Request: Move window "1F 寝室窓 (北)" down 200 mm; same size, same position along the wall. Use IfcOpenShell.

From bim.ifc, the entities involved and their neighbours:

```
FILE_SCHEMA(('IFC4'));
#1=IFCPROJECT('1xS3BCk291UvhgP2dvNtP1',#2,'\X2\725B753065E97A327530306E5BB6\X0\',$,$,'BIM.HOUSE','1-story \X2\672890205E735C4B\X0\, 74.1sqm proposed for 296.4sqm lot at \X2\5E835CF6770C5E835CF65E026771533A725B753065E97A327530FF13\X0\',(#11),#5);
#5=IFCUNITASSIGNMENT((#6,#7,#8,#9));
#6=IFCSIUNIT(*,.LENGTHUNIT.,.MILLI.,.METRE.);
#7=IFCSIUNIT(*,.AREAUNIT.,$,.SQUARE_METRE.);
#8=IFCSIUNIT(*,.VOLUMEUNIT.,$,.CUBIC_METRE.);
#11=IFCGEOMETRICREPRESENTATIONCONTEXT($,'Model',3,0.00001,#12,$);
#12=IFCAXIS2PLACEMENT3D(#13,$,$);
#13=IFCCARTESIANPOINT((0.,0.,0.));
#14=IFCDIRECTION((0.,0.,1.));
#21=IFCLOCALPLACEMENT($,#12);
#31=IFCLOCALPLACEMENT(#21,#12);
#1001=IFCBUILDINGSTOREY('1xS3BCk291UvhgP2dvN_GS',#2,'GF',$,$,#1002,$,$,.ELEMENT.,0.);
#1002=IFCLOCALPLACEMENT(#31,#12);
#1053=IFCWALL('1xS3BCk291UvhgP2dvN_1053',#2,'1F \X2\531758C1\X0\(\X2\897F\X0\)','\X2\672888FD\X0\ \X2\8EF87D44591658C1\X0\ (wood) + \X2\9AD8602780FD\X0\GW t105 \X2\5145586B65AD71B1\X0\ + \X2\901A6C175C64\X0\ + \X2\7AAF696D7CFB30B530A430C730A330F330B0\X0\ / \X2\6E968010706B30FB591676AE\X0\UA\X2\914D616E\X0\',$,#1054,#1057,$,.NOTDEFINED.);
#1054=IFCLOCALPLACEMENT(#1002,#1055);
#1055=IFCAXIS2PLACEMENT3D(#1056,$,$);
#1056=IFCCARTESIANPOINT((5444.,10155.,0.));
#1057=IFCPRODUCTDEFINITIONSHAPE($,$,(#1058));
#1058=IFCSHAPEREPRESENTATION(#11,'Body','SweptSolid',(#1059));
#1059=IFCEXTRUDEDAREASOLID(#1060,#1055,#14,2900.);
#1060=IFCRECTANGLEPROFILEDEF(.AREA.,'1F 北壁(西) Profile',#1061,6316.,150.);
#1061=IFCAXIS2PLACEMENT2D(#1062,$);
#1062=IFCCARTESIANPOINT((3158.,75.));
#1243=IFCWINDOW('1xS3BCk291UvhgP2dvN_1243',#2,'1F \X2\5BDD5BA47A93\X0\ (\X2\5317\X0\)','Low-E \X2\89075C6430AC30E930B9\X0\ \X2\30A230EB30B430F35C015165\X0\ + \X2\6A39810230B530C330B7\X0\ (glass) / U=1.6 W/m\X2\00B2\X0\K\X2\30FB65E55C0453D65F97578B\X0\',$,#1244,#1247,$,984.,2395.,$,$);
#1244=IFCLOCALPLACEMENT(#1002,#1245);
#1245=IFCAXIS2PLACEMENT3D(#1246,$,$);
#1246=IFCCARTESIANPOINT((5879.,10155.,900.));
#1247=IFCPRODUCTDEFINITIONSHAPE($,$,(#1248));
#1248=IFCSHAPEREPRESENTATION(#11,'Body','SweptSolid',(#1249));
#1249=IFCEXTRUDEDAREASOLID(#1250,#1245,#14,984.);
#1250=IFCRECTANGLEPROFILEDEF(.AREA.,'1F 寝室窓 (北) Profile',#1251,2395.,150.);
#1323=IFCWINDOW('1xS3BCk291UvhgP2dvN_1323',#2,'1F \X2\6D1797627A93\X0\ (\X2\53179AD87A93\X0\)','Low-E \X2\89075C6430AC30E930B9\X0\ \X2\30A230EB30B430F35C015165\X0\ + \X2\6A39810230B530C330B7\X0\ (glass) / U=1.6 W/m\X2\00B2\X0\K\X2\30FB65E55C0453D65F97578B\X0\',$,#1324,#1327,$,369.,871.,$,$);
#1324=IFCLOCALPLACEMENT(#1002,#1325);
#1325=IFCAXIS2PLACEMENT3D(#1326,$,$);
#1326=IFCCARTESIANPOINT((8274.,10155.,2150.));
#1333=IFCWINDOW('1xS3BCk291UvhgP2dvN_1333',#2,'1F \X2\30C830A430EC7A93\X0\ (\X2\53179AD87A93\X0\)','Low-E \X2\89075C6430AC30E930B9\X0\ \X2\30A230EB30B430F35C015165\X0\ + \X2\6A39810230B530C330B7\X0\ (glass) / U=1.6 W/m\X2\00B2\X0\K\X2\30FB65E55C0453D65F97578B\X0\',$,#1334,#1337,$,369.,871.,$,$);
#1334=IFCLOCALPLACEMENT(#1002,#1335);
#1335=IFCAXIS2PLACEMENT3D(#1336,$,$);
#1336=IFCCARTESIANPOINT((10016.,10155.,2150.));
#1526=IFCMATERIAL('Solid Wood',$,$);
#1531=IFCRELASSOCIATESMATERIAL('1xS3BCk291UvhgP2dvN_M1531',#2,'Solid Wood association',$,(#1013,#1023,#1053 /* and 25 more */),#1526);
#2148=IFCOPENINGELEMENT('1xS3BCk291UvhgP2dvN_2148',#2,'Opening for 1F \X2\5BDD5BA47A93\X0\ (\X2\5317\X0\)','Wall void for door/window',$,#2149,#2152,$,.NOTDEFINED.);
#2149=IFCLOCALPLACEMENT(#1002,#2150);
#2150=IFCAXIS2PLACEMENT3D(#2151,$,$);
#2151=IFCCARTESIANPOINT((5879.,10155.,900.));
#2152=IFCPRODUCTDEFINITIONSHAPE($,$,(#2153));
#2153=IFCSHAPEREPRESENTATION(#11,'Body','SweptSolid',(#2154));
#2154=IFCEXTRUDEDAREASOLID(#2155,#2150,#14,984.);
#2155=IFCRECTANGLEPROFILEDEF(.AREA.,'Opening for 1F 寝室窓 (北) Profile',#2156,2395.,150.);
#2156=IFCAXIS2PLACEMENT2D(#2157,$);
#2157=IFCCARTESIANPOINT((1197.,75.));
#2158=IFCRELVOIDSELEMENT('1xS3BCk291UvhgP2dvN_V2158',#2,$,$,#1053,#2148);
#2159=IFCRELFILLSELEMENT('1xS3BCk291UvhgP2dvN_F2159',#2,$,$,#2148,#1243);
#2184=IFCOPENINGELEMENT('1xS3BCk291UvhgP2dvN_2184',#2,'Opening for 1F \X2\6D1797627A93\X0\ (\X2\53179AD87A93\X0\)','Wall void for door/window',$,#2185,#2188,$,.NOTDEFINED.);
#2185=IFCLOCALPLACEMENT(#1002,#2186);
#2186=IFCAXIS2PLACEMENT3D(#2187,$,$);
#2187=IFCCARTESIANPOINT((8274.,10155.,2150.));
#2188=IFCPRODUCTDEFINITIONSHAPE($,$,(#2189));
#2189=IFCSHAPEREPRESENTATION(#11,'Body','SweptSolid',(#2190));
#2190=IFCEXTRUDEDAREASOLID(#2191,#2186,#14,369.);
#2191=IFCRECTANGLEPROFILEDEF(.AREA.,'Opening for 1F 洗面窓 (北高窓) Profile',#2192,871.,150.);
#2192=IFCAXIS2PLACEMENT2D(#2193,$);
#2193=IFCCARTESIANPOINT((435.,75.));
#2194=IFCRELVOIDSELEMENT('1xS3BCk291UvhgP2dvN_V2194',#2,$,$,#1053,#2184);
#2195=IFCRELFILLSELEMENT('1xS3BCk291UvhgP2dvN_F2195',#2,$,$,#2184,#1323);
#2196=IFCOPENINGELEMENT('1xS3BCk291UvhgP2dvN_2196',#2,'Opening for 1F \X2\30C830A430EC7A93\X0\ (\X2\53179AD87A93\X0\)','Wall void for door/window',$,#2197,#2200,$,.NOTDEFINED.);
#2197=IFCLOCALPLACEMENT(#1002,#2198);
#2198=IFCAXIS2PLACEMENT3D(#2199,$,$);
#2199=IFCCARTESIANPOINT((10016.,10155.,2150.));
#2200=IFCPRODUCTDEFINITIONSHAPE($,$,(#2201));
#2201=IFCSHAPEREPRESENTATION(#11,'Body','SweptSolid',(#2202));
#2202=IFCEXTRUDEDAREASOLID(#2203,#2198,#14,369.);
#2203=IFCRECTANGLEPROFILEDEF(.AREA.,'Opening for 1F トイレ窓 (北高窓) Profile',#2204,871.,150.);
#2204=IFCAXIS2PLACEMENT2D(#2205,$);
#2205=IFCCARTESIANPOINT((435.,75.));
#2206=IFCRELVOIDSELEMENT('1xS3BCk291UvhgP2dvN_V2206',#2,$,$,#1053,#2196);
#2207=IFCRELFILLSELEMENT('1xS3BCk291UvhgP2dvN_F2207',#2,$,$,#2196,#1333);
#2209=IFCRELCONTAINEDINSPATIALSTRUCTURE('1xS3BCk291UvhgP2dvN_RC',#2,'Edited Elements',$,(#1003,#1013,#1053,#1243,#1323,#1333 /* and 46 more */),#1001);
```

```python
import numpy as np
import ifcopenshell
import ifcopenshell.api.geometry
import ifcopenshell.util.placement
import ifcopenshell.util.unit

model = ifcopenshell.open("bim.ifc")
unit_scale = ifcopenshell.util.unit.calculate_unit_scale(model)

window = model.by_guid("1xS3BCk291UvhgP2dvN_1243")
opening = window.FillsVoids[0].RelatingOpeningElement
dz = -0.2 / unit_scale

shift = np.array([0.0, 0.0, dz])
# The window is not placed relative to its opening, so move both.
for product in (opening, window):
    matrix = ifcopenshell.util.placement.get_local_placement(product.ObjectPlacement)
    matrix[:3, 3] += shift
    ifcopenshell.api.geometry.edit_object_placement(model, product=product, matrix=matrix, is_si=False)

print(f"moved by {dz * unit_scale:+.3f} m")

model.write("bim-out.ifc")
```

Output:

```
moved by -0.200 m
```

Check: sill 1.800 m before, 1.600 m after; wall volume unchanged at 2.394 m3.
